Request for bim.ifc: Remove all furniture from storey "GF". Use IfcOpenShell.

First a look at what the model holds.

```python
import ifcopenshell
import ifcopenshell.util.element

model = ifcopenshell.open("bim.ifc")
print(model.schema)
storey = next(s for s in model.by_type("IfcBuildingStorey") if s.Name == "GF")
furniture = [e for e in ifcopenshell.util.element.get_decomposition(storey) if e.is_a("IfcFurnishingElement")]
seen = {}
for e in furniture:
    element_type = ifcopenshell.util.element.get_type(e)
    name = element_type.Name if element_type not in (None, e) else None
    seen[name] = seen.get(name, 0) + 1
for name, count in sorted(seen.items(), key=str):
    print(count, "x", name)
```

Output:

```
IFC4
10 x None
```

```python
import ifcopenshell
import ifcopenshell.api.root
import ifcopenshell.util.element

model = ifcopenshell.open("bim.ifc")

storey = next(s for s in model.by_type("IfcBuildingStorey") if s.Name == "GF")
furniture = [e for e in ifcopenshell.util.element.get_decomposition(storey) if e.is_a("IfcFurnishingElement")]

for e in furniture:
    ifcopenshell.api.root.remove_product(model, product=e)
print(len(furniture), "removed")

model.write("bim_updated.ifc")
```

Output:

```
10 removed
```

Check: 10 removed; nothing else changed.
